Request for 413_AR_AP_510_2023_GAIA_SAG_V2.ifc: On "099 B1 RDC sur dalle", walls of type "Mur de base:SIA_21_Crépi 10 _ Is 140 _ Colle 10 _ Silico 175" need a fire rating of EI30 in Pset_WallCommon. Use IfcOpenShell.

First a look at what the model holds.

```python
import ifcopenshell
import ifcopenshell.util.element

model = ifcopenshell.open("413_AR_AP_510_2023_GAIA_SAG_V2.ifc")
print(model.schema)
storey = next(s for s in model.by_type("IfcBuildingStorey") if s.Name == "099 B1 RDC sur dalle")
walls = [e for e in ifcopenshell.util.element.get_decomposition(storey) if e.is_a("IfcWall")]
seen = {}
for e in walls:
    element_type = ifcopenshell.util.element.get_type(e)
    key = (element_type.Name if element_type != e and element_type else None, ifcopenshell.util.element.get_pset(e, "Pset_WallCommon", "FireRating"))
    seen[key] = seen.get(key, 0) + 1
for (name, value), count in sorted(seen.items(), key=str):
    print(count, "x", name, "|", value)
```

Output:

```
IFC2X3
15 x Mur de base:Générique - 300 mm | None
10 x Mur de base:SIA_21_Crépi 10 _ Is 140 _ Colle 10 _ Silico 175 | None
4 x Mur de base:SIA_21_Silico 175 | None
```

```python
import ifcopenshell
import ifcopenshell.api.pset
import ifcopenshell.util.element

model = ifcopenshell.open("413_AR_AP_510_2023_GAIA_SAG_V2.ifc")

storey = next(s for s in model.by_type("IfcBuildingStorey") if s.Name == "099 B1 RDC sur dalle")
walls = [e for e in ifcopenshell.util.element.get_decomposition(storey) if e.is_a("IfcWall")]

count = 0
for e in walls:
    element_type = ifcopenshell.util.element.get_type(e)
    if element_type in (None, e) or element_type.Name != "Mur de base:SIA_21_Crépi 10 _ Is 140 _ Colle 10 _ Silico 175":
        continue
    # add_pset returns the element's existing set when there is one.
    pset = ifcopenshell.api.pset.add_pset(model, product=e, name="Pset_WallCommon")
    ifcopenshell.api.pset.edit_pset(model, pset=pset, properties={"FireRating": "EI30"})
    count += 1

print(count, "walls updated")

model.write("413_AR_AP_510_2023_GAIA_SAG_V2_rev.ifc")
```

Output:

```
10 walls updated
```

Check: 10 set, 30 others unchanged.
